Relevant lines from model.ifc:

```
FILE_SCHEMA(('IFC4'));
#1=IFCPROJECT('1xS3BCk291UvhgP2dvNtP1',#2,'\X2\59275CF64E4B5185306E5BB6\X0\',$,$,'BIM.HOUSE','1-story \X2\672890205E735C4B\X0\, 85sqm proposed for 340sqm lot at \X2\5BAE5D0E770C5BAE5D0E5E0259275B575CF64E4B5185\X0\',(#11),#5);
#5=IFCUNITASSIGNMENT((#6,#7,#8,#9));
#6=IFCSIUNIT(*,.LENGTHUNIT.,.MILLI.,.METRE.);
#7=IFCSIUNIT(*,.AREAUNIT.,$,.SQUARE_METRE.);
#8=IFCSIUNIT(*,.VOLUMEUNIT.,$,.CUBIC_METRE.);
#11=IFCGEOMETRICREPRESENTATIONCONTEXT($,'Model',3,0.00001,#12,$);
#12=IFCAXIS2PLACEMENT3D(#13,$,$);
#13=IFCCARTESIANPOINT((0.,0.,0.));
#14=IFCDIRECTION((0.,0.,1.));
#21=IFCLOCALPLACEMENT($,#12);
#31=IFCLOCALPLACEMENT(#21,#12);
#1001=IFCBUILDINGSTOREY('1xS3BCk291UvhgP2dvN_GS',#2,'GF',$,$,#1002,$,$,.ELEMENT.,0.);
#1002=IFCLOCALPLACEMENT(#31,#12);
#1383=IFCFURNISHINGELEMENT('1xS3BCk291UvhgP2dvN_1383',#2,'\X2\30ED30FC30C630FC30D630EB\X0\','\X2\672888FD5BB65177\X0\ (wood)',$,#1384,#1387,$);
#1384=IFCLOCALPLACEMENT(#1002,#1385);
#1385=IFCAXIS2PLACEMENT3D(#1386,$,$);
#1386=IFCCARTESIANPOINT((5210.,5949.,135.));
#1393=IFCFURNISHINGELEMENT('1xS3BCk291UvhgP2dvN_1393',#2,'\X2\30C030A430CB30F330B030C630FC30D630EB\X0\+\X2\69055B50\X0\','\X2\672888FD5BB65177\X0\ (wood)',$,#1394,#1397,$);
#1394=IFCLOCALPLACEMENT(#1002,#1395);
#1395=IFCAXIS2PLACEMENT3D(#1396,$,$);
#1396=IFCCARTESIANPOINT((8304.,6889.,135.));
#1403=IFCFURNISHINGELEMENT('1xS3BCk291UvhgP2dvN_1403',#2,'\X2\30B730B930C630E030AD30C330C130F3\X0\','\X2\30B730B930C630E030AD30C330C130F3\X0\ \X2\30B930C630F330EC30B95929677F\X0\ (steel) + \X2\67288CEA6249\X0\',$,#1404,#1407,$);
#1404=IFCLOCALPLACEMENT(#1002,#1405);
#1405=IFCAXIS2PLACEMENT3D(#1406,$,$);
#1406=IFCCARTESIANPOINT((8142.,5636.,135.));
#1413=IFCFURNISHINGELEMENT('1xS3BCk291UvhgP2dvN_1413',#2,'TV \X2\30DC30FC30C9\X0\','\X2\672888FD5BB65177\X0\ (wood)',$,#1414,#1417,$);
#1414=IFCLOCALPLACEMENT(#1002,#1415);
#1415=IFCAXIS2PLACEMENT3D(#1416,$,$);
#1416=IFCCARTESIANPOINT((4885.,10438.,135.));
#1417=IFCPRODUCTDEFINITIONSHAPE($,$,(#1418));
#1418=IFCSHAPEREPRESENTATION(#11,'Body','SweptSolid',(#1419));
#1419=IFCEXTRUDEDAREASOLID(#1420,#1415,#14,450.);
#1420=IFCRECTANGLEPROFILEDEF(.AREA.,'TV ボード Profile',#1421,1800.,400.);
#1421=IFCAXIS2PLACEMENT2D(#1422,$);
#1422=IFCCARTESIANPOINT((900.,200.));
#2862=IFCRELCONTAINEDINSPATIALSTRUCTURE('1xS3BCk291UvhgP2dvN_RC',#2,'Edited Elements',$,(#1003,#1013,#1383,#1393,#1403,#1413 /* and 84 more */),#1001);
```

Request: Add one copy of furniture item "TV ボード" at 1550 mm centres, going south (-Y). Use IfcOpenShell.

```python
import numpy as np
import ifcopenshell
import ifcopenshell.api.geometry
import ifcopenshell.api.root
import ifcopenshell.util.element
import ifcopenshell.util.placement
import ifcopenshell.util.unit

model = ifcopenshell.open("model.ifc")
unit_scale = ifcopenshell.util.unit.calculate_unit_scale(model)


def reuse_history(source, copy):
    """copy_class also copies each property set's owner history, people and application; keep the originals."""
    for rel in copy.IsDefinedBy:
        if rel.is_a("IfcRelDefinesByProperties") and (history := rel.RelatingPropertyDefinition.OwnerHistory):
            rel.RelatingPropertyDefinition.OwnerHistory = source.OwnerHistory
            ifcopenshell.util.element.remove_deep2(model, history)


source = model.by_guid("1xS3BCk291UvhgP2dvN_1413")
base = ifcopenshell.util.placement.get_local_placement(source.ObjectPlacement)
step = np.array([0.0, -1.0, 0.0]) * 1.55 / unit_scale

for i in range(1, 2):
    copy = ifcopenshell.api.root.copy_class(model, product=source)
    copy.Representation = ifcopenshell.util.element.copy_deep(
        model, source.Representation, exclude=["IfcGeometricRepresentationContext", "IfcRepresentationMap"]
    )
    reuse_history(source, copy)
    matrix = base.copy()
    matrix[:3, 3] += i * step
    print("added at", matrix[:3, 3].round(3) + 0.0)
    ifcopenshell.api.geometry.edit_object_placement(model, product=copy, matrix=matrix, is_si=False)

model.write("model_rev.ifc")
```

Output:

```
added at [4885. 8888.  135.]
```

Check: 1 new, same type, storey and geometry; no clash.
